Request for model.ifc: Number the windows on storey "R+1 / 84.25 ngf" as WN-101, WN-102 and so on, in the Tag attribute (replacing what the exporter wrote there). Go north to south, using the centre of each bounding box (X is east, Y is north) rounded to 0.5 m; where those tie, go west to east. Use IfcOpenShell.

First a look at what the model holds.

```python
import ifcopenshell
import ifcopenshell.util.element
import ifcopenshell.util.placement

model = ifcopenshell.open("model.ifc")
print(model.schema)
storey = next(s for s in model.by_type("IfcBuildingStorey") if s.Name == "R+1 / 84.25 ngf")
windows = [e for e in ifcopenshell.util.element.get_decomposition(storey) if e.is_a("IfcWindow")]
for e in sorted(windows, key=lambda e: e.id()):
    origin = ifcopenshell.util.placement.get_local_placement(e.ObjectPlacement)[:3, 3]
    print(e.id(), e.Tag, e.Name, origin.round(2) + 0.0, sep=" | ")
```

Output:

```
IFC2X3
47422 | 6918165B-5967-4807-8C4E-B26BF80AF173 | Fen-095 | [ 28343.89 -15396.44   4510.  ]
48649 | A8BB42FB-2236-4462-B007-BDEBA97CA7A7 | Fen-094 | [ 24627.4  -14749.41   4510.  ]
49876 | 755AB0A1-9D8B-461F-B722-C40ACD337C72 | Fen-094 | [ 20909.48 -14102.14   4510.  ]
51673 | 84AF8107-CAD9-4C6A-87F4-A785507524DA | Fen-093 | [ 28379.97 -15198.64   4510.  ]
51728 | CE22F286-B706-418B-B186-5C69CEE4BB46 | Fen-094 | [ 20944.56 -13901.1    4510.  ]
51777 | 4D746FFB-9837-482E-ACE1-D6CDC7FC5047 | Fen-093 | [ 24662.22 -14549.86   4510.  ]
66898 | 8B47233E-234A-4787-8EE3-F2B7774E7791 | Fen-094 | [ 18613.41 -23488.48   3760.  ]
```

```python
import ifcopenshell
import ifcopenshell.geom
import ifcopenshell.util.element
import ifcopenshell.util.shape

model = ifcopenshell.open("model.ifc")
settings = ifcopenshell.geom.settings()
settings.set("use-world-coords", True)


def centre(element):
    shape = ifcopenshell.geom.create_shape(settings, element)
    return ifcopenshell.util.shape.get_bbox_centroid(shape.geometry)


storey = next(s for s in model.by_type("IfcBuildingStorey") if s.Name == "R+1 / 84.25 ngf")
windows = [e for e in ifcopenshell.util.element.get_decomposition(storey) if e.is_a("IfcWindow")]

# Insertion points can sit at a corner or the storey origin, so sort by the geometry (in metres).
centres = {e: centre(e) for e in windows}
windows.sort(key=lambda e: (-round(centres[e][1] / 0.5), centres[e][0]))

for i, e in enumerate(windows, start=1):
    number = f"WN-1{i:02d}"
    e.Tag = number
    print(e.id(), number)

model.write("model_v2.ifc")
```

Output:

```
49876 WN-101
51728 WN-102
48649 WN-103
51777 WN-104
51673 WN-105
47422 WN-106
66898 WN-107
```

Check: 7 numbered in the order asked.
